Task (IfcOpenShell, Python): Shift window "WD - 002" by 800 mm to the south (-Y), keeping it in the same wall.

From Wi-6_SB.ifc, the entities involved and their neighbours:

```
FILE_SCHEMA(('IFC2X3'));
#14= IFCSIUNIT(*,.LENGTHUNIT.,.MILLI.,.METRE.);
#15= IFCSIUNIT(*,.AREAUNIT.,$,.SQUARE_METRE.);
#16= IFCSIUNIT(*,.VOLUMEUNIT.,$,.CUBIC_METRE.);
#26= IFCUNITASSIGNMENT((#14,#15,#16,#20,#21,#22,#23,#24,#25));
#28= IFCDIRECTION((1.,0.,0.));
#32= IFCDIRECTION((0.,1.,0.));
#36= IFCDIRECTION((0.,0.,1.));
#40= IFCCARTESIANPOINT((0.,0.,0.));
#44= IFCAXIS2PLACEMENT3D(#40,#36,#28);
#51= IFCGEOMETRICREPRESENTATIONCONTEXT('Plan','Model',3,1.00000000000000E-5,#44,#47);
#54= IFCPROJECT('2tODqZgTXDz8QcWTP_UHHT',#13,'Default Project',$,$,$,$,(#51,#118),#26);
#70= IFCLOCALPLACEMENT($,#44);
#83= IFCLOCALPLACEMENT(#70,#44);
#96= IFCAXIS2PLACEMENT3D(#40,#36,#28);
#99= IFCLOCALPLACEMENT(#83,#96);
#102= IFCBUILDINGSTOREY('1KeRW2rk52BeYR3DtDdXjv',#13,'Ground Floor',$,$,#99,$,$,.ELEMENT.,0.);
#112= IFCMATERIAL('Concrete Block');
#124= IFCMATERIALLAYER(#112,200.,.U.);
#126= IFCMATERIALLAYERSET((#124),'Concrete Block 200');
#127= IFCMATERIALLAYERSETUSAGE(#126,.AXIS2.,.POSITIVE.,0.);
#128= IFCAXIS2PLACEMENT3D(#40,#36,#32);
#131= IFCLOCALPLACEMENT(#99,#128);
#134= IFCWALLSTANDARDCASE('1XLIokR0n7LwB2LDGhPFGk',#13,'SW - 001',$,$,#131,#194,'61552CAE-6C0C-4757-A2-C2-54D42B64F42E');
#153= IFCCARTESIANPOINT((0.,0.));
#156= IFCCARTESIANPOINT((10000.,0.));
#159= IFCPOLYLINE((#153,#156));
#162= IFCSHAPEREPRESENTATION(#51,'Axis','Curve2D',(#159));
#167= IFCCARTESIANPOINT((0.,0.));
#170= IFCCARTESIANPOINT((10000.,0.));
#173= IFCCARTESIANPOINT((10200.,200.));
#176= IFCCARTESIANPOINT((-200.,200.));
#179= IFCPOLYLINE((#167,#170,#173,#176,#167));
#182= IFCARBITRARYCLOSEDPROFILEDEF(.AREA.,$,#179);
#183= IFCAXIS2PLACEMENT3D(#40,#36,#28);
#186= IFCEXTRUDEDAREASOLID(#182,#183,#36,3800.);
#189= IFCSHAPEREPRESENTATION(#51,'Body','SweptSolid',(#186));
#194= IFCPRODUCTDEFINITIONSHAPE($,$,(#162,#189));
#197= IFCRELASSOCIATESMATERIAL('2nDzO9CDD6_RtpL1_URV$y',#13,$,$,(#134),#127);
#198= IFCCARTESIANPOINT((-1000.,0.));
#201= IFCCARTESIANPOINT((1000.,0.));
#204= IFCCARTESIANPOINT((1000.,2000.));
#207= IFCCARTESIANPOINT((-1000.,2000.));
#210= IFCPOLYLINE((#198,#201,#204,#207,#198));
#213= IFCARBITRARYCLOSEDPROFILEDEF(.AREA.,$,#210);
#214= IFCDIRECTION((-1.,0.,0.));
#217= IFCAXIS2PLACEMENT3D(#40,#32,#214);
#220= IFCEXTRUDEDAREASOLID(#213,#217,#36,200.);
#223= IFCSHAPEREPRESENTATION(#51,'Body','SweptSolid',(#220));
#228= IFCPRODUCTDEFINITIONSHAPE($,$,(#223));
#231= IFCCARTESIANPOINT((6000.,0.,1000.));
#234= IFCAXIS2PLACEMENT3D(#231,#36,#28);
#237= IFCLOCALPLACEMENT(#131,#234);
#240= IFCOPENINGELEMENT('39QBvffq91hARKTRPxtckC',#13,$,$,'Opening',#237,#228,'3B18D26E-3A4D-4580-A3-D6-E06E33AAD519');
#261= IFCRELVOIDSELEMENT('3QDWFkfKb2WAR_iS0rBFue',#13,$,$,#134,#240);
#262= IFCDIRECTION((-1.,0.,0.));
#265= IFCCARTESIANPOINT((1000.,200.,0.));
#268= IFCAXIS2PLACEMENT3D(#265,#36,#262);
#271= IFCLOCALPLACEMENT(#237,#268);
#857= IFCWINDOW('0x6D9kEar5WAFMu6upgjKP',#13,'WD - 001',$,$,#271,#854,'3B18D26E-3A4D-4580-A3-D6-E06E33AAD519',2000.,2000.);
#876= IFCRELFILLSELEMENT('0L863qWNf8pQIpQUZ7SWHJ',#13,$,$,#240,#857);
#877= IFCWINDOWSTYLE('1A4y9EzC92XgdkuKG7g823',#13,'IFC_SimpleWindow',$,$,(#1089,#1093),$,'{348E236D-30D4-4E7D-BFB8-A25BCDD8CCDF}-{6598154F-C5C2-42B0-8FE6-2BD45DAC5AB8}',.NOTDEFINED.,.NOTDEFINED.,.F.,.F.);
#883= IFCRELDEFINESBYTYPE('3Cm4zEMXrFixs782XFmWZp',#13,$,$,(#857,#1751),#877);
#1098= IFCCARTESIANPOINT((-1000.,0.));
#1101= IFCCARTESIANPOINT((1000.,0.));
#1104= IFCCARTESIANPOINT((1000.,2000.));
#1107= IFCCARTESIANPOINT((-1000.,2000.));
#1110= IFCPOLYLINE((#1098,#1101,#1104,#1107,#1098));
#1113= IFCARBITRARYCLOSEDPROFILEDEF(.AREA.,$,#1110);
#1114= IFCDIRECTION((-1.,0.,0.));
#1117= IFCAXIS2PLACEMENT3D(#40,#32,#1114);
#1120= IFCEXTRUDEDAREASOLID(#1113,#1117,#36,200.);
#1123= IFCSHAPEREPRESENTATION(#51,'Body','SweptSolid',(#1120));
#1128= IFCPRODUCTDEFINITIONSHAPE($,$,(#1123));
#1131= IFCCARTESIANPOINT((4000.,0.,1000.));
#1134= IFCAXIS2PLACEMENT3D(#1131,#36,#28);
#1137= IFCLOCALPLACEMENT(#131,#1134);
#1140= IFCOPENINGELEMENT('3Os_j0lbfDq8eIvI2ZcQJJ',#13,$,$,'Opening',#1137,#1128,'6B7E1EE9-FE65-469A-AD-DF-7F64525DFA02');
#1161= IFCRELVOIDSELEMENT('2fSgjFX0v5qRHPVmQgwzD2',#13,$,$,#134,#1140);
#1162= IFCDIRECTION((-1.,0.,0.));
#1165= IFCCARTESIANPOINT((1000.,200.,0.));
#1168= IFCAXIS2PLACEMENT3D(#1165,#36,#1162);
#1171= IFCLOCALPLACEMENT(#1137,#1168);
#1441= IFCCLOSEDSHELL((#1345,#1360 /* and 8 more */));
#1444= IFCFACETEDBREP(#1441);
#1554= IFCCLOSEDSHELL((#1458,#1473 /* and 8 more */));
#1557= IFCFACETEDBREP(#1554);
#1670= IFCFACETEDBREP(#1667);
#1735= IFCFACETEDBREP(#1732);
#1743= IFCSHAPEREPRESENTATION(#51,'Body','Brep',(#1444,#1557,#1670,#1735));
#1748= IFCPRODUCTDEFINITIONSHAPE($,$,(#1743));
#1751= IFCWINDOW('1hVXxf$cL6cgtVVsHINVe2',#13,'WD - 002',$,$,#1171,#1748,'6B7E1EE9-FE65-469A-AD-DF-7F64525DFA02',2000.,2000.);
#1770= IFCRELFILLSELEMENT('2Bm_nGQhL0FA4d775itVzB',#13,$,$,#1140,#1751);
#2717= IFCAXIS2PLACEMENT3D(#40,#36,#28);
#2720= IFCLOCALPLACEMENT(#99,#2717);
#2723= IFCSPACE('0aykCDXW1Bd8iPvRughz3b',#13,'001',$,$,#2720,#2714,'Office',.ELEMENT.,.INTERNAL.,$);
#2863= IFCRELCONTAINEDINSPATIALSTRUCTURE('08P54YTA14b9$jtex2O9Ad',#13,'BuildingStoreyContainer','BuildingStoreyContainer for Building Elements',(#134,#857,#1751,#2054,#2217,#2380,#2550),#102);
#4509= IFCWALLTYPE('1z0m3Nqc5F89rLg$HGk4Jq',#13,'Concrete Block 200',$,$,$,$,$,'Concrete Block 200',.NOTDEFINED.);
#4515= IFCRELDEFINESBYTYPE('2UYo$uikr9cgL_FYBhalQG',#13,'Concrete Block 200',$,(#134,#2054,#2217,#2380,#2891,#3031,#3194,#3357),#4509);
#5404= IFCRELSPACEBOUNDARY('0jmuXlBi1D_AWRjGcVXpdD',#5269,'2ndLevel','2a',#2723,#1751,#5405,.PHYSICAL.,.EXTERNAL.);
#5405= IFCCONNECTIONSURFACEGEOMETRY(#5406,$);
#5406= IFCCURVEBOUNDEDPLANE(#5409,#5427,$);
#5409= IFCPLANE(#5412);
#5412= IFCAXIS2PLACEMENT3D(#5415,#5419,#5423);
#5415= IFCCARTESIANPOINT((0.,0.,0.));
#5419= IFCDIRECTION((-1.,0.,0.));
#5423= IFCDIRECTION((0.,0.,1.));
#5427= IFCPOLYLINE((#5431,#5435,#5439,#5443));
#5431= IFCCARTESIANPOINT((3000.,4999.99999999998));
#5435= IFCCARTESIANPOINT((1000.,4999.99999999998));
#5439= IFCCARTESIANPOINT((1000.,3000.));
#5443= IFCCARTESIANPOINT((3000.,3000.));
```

```python
import numpy as np
import ifcopenshell
import ifcopenshell.api.geometry
import ifcopenshell.util.placement
import ifcopenshell.util.unit

model = ifcopenshell.open("Wi-6_SB.ifc")
unit_scale = ifcopenshell.util.unit.calculate_unit_scale(model)

window = model.by_guid("1hVXxf$cL6cgtVVsHINVe2")
opening = window.FillsVoids[0].RelatingOpeningElement
wall = opening.VoidsElements[0].RelatingBuildingElement

wall_matrix = ifcopenshell.util.placement.get_local_placement(wall.ObjectPlacement)
shift = wall_matrix[:3, 0] * -0.8 / unit_scale
before = ifcopenshell.util.placement.get_local_placement(window.ObjectPlacement)[:3, 3].copy()

# The window is placed relative to its opening, so it follows when the opening moves.
matrix = ifcopenshell.util.placement.get_local_placement(opening.ObjectPlacement)
matrix[:3, 3] += shift
ifcopenshell.api.geometry.edit_object_placement(
    model, product=opening, matrix=matrix, is_si=False, should_transform_children=True
)

# Space boundary surfaces are stored in each space's coordinates; move them too.
for rel in window.ProvidesBoundaries:
    if not rel.ConnectionGeometry:
        continue
    surface = rel.ConnectionGeometry.SurfaceOnRelatingElement.BasisSurface
    space_matrix = ifcopenshell.util.placement.get_local_placement(rel.RelatingSpace.ObjectPlacement)
    point = np.array(surface.Position.Location.Coordinates) + space_matrix[:3, :3].T @ shift
    surface.Position = model.createIfcAxis2Placement3D(
        model.createIfcCartesianPoint(point.tolist()), surface.Position.Axis, surface.Position.RefDirection
    )

after = ifcopenshell.util.placement.get_local_placement(window.ObjectPlacement)[:3, 3]
print("window moved by", (after - before).round(3) + 0.0)

model.write("Wi-6_SB_updated.ifc")
```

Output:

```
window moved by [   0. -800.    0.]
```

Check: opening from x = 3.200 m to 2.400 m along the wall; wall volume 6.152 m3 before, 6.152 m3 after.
